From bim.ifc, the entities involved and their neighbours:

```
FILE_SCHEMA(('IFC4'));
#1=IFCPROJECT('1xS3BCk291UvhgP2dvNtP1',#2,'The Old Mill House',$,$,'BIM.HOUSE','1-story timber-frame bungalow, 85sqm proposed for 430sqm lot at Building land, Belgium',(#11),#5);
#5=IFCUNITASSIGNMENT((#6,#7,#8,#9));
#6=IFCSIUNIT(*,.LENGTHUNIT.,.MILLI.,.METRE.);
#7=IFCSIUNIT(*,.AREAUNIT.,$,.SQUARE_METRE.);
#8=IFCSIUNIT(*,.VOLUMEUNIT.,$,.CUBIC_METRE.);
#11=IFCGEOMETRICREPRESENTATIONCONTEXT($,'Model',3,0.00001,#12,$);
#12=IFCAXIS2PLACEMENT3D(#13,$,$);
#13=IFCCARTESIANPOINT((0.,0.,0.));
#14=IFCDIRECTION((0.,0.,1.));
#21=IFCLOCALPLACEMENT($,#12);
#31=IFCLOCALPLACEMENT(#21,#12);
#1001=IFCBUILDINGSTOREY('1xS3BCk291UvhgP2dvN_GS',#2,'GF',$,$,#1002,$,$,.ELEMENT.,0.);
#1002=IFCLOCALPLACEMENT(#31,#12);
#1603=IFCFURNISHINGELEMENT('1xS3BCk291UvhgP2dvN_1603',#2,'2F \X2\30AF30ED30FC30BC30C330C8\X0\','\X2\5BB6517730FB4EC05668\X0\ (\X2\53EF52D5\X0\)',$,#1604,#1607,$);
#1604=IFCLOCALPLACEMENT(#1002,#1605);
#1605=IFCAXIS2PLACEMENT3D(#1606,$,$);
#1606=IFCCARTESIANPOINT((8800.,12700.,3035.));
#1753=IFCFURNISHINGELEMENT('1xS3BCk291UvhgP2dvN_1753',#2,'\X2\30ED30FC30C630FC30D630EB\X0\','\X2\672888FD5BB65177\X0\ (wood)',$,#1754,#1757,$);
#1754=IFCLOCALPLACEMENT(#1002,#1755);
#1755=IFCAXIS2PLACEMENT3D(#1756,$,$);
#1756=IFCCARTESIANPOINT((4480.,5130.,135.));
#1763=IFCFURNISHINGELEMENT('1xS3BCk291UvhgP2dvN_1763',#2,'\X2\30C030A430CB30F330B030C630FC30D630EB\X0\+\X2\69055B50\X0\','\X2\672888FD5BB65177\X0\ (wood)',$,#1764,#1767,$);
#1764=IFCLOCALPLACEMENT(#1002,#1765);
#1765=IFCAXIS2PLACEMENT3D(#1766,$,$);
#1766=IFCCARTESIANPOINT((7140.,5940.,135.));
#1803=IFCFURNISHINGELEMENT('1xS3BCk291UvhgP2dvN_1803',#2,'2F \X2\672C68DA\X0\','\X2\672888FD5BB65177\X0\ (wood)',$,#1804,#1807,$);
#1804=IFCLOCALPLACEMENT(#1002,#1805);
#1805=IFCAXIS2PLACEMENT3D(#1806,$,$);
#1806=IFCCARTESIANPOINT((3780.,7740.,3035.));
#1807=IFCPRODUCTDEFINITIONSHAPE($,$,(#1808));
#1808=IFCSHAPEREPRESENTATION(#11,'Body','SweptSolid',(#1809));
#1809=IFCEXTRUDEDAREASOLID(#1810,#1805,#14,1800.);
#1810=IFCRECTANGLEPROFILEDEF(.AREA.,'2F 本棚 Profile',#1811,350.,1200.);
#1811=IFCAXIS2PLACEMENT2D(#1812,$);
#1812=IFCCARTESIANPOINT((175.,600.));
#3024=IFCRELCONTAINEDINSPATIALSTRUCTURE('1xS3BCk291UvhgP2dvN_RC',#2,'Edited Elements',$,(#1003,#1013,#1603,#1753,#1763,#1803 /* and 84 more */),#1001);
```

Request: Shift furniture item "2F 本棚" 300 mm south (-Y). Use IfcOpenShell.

```python
import ifcopenshell
import ifcopenshell.api.geometry
import ifcopenshell.util.placement
import ifcopenshell.util.unit

model = ifcopenshell.open("bim.ifc")
unit_scale = ifcopenshell.util.unit.calculate_unit_scale(model)

item = model.by_guid("1xS3BCk291UvhgP2dvN_1803")
matrix = ifcopenshell.util.placement.get_local_placement(item.ObjectPlacement)
matrix[1, 3] -= 0.3 / unit_scale
ifcopenshell.api.geometry.edit_object_placement(model, product=item, matrix=matrix, is_si=False)

print(ifcopenshell.util.placement.get_local_placement(item.ObjectPlacement).round(3) + 0.0)

model.write("bim-out.ifc")
```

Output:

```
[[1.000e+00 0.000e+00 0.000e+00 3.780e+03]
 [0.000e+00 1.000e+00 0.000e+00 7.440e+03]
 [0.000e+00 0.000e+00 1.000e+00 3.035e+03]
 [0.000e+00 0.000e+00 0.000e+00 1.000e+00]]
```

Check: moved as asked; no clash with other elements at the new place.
